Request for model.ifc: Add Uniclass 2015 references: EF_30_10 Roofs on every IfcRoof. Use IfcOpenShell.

First a look at what the model holds.

```python
import ifcopenshell

model = ifcopenshell.open("model.ifc")
print(model.schema)
print("classifications:", [c.Name for c in model.by_type("IfcClassification")])
for ifc_class in ("IfcDoor", "IfcRoof", "IfcStair", "IfcWall", "IfcWindow"):
    print(ifc_class, len(model.by_type(ifc_class)))
```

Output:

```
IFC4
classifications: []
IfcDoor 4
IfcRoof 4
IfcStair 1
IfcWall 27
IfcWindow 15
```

```python
import ifcopenshell
import ifcopenshell.api.classification

model = ifcopenshell.open("model.ifc")

system = ifcopenshell.api.classification.add_classification(model, classification="Uniclass 2015")

codes = {
    "IfcRoof": ("EF_30_10", "Roofs"),
}
for ifc_class, (code, name) in codes.items():
    products = model.by_type(ifc_class)
    ifcopenshell.api.classification.add_reference(
        model, products=products, classification=system, identification=code, name=name
    )
    print(code, len(products))

model.write("model_edited.ifc")
```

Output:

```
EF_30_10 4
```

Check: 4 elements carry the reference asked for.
